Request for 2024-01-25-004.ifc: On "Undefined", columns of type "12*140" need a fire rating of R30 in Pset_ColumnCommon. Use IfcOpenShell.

First a look at what the model holds.

```python
import ifcopenshell
import ifcopenshell.util.element

model = ifcopenshell.open("2024-01-25-004.ifc")
print(model.schema)
storey = next(s for s in model.by_type("IfcBuildingStorey") if s.Name == "Undefined")
columns = [e for e in ifcopenshell.util.element.get_decomposition(storey) if e.is_a("IfcColumn")]
seen = {}
for e in columns:
    element_type = ifcopenshell.util.element.get_type(e)
    key = (element_type.Name if element_type != e and element_type else None, ifcopenshell.util.element.get_pset(e, "Pset_ColumnCommon", "FireRating"))
    seen[key] = seen.get(key, 0) + 1
for (name, value), count in sorted(seen.items(), key=str):
    print(count, "x", name, "|", value)
```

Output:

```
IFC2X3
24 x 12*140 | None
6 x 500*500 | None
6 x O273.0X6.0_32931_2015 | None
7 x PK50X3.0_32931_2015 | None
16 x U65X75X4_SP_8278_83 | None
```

```python
import ifcopenshell
import ifcopenshell.api.pset
import ifcopenshell.util.element

model = ifcopenshell.open("2024-01-25-004.ifc")

storey = next(s for s in model.by_type("IfcBuildingStorey") if s.Name == "Undefined")
columns = [e for e in ifcopenshell.util.element.get_decomposition(storey) if e.is_a("IfcColumn")]

count = 0
for e in columns:
    element_type = ifcopenshell.util.element.get_type(e)
    if element_type in (None, e) or element_type.Name != "12*140":
        continue
    found = ifcopenshell.util.element.get_pset(e, "Pset_ColumnCommon", should_inherit=False)
    if found:
        pset = model.by_id(found["id"])
        if len(ifcopenshell.util.element.get_elements_by_pset(pset)) > 1:
            pset = ifcopenshell.api.pset.unshare_pset(model, products=[e], pset=pset)[0]
    else:
        pset = ifcopenshell.api.pset.add_pset(model, product=e, name="Pset_ColumnCommon")
    ifcopenshell.api.pset.edit_pset(model, pset=pset, properties={"FireRating": "R30"})
    count += 1

print(count, "columns updated")

model.write("2024-01-25-004_updated.ifc")
```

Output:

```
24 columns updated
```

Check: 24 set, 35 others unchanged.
